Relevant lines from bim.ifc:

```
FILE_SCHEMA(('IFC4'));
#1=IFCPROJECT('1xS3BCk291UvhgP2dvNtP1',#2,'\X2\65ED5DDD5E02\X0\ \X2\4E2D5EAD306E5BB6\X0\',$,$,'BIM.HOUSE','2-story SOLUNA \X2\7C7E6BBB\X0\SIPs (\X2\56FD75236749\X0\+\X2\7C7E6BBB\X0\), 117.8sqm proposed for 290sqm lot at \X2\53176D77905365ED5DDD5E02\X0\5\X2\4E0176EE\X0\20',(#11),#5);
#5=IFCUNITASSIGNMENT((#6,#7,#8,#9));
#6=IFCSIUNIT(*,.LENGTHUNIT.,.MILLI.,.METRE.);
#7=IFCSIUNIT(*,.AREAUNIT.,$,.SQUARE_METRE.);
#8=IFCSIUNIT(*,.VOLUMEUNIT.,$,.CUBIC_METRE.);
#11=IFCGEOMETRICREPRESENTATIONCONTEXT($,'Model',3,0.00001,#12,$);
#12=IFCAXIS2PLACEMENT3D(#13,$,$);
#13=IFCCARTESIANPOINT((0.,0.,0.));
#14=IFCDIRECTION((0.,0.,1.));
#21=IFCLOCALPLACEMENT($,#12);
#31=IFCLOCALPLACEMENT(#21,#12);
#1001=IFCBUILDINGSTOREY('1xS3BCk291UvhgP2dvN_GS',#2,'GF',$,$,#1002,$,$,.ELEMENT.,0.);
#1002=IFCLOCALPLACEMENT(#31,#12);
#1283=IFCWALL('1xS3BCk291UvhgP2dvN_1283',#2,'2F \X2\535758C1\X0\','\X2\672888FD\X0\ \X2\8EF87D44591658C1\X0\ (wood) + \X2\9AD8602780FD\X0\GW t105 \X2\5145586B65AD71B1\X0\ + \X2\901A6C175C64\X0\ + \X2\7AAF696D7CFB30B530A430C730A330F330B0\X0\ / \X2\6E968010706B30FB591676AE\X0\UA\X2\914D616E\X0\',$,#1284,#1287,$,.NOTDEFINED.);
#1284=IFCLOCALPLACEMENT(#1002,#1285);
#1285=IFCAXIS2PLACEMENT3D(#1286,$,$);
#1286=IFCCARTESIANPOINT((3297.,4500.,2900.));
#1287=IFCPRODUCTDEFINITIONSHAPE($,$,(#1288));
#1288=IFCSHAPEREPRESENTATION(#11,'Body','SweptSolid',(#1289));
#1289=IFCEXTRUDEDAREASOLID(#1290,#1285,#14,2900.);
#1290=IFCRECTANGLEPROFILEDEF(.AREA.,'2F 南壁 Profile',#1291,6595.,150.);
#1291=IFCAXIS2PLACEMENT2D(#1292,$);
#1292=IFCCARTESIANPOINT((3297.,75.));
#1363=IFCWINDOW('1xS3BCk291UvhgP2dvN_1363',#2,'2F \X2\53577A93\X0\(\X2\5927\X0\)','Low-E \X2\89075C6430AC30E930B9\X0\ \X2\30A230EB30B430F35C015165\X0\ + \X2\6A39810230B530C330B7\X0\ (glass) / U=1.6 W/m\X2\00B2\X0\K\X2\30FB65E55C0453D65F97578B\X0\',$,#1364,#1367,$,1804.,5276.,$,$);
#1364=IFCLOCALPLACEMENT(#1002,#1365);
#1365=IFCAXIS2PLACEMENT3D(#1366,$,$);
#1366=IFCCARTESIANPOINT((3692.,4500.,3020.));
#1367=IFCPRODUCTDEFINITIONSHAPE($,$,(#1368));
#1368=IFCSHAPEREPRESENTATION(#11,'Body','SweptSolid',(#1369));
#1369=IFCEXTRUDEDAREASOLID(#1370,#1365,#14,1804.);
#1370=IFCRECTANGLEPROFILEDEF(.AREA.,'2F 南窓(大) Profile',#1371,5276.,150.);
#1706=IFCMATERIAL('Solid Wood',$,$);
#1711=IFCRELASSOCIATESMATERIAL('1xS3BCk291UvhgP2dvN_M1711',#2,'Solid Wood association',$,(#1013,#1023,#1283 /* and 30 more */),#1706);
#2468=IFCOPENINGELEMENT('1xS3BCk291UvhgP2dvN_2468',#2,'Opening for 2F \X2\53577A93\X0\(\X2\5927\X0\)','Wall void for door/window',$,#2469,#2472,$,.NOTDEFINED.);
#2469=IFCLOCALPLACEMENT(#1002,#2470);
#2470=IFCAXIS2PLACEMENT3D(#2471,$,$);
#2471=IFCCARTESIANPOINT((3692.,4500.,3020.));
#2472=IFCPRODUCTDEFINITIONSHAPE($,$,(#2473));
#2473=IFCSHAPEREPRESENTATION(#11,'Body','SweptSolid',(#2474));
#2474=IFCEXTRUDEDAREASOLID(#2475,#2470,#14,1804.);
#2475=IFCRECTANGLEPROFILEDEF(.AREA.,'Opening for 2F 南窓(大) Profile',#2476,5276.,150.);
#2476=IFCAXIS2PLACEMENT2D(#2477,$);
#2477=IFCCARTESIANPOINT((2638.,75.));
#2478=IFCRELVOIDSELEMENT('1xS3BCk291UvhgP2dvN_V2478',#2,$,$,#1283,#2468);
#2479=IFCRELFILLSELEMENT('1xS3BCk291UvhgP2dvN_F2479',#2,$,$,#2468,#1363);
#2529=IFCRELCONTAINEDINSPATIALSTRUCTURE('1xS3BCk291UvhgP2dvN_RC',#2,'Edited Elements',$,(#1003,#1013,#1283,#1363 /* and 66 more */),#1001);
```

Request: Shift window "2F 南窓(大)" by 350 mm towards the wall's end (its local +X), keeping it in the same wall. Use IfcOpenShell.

```python
import ifcopenshell
import ifcopenshell.api.geometry
import ifcopenshell.util.placement

model = ifcopenshell.open("bim.ifc")

window = model.by_id(1363)
opening = window.FillsVoids[0].RelatingOpeningElement
wall = opening.VoidsElements[0].RelatingBuildingElement

wall_matrix = ifcopenshell.util.placement.get_local_placement(wall.ObjectPlacement)
shift = wall_matrix[:3, 0] * 350.0
before = ifcopenshell.util.placement.get_local_placement(window.ObjectPlacement)[:3, 3].copy()

# The window is not placed relative to its opening, so move both.
for product in (opening, window):
    matrix = ifcopenshell.util.placement.get_local_placement(product.ObjectPlacement)
    matrix[:3, 3] += shift
    ifcopenshell.api.geometry.edit_object_placement(model, product=product, matrix=matrix, is_si=False)

after = ifcopenshell.util.placement.get_local_placement(window.ObjectPlacement)[:3, 3]
print("window moved by", (after - before).round(3) + 0.0)

model.write("bim_rev.ifc")
```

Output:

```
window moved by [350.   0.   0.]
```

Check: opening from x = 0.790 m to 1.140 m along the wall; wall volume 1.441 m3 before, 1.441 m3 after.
